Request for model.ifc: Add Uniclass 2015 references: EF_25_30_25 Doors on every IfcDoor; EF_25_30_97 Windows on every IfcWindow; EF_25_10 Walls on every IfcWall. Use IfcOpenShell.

First a look at what the model holds.

```python
import ifcopenshell

model = ifcopenshell.open("model.ifc")
print(model.schema)
print("classifications:", [c.Name for c in model.by_type("IfcClassification")])
for ifc_class in ("IfcDoor", "IfcRoof", "IfcStair", "IfcWall", "IfcWindow"):
    print(ifc_class, len(model.by_type(ifc_class)))
```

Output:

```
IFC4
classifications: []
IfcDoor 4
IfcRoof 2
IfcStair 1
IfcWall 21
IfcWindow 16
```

```python
import ifcopenshell
import ifcopenshell.api.classification

model = ifcopenshell.open("model.ifc")

system = ifcopenshell.api.classification.add_classification(model, classification="Uniclass 2015")

codes = {
    "IfcDoor": ("EF_25_30_25", "Doors"),
    "IfcWindow": ("EF_25_30_97", "Windows"),
    "IfcWall": ("EF_25_10", "Walls"),
}
for ifc_class, (code, name) in codes.items():
    products = model.by_type(ifc_class)
    ifcopenshell.api.classification.add_reference(
        model, products=products, classification=system, identification=code, name=name
    )
    print(code, len(products))

model.write("model-out.ifc")
```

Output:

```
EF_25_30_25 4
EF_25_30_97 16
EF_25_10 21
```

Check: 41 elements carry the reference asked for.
